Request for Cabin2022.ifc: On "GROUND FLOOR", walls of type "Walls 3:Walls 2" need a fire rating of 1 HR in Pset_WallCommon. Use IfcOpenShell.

First a look at what the model holds.

```python
import ifcopenshell
import ifcopenshell.util.element

model = ifcopenshell.open("Cabin2022.ifc")
print(model.schema)
storey = next(s for s in model.by_type("IfcBuildingStorey") if s.Name == "GROUND FLOOR")
walls = [e for e in ifcopenshell.util.element.get_decomposition(storey) if e.is_a("IfcWall")]
seen = {}
for e in walls:
    element_type = ifcopenshell.util.element.get_type(e)
    key = (element_type.Name if element_type != e and element_type else None, ifcopenshell.util.element.get_pset(e, "Pset_WallCommon", "FireRating"))
    seen[key] = seen.get(key, 0) + 1
for (name, value), count in sorted(seen.items(), key=str):
    print(count, "x", name, "|", value)
```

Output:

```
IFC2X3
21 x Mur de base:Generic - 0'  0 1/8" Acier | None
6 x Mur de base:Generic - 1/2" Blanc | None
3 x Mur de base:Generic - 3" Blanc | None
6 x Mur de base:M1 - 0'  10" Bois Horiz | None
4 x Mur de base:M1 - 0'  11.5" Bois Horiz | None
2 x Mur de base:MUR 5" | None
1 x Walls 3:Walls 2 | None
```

```python
import ifcopenshell
import ifcopenshell.api.pset
import ifcopenshell.util.element

model = ifcopenshell.open("Cabin2022.ifc")

storey = next(s for s in model.by_type("IfcBuildingStorey") if s.Name == "GROUND FLOOR")
walls = [e for e in ifcopenshell.util.element.get_decomposition(storey) if e.is_a("IfcWall")]

count = 0
for e in walls:
    element_type = ifcopenshell.util.element.get_type(e)
    if element_type in (None, e) or element_type.Name != "Walls 3:Walls 2":
        continue
    # add_pset returns the element's existing set when there is one.
    pset = ifcopenshell.api.pset.add_pset(model, product=e, name="Pset_WallCommon")
    ifcopenshell.api.pset.edit_pset(model, pset=pset, properties={"FireRating": "1 HR"})
    count += 1

print(count, "walls updated")

model.write("Cabin2022_v2.ifc")
```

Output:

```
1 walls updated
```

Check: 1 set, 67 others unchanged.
